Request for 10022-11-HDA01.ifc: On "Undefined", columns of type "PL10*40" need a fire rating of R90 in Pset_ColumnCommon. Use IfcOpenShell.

First a look at what the model holds.

```python
import ifcopenshell
import ifcopenshell.util.element

model = ifcopenshell.open("10022-11-HDA01.ifc")
print(model.schema)
storey = next(s for s in model.by_type("IfcBuildingStorey") if s.Name == "Undefined")
columns = [e for e in ifcopenshell.util.element.get_decomposition(storey) if e.is_a("IfcColumn")]
seen = {}
for e in columns:
    element_type = ifcopenshell.util.element.get_type(e)
    key = (element_type.Name if element_type != e and element_type else None, ifcopenshell.util.element.get_pset(e, "Pset_ColumnCommon", "FireRating"))
    seen[key] = seen.get(key, 0) + 1
for (name, value), count in sorted(seen.items(), key=str):
    print(count, "x", name, "|", value)
```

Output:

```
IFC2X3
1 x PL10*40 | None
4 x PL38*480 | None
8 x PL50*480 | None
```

```python
import ifcopenshell
import ifcopenshell.api.pset
import ifcopenshell.util.element

model = ifcopenshell.open("10022-11-HDA01.ifc")

storey = next(s for s in model.by_type("IfcBuildingStorey") if s.Name == "Undefined")
columns = [e for e in ifcopenshell.util.element.get_decomposition(storey) if e.is_a("IfcColumn")]

count = 0
for e in columns:
    element_type = ifcopenshell.util.element.get_type(e)
    if element_type in (None, e) or element_type.Name != "PL10*40":
        continue
    # add_pset returns the element's existing set when there is one.
    pset = ifcopenshell.api.pset.add_pset(model, product=e, name="Pset_ColumnCommon")
    ifcopenshell.api.pset.edit_pset(model, pset=pset, properties={"FireRating": "R90"})
    count += 1

print(count, "columns updated")

model.write("10022-11-HDA01_rev.ifc")
```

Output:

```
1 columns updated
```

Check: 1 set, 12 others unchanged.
